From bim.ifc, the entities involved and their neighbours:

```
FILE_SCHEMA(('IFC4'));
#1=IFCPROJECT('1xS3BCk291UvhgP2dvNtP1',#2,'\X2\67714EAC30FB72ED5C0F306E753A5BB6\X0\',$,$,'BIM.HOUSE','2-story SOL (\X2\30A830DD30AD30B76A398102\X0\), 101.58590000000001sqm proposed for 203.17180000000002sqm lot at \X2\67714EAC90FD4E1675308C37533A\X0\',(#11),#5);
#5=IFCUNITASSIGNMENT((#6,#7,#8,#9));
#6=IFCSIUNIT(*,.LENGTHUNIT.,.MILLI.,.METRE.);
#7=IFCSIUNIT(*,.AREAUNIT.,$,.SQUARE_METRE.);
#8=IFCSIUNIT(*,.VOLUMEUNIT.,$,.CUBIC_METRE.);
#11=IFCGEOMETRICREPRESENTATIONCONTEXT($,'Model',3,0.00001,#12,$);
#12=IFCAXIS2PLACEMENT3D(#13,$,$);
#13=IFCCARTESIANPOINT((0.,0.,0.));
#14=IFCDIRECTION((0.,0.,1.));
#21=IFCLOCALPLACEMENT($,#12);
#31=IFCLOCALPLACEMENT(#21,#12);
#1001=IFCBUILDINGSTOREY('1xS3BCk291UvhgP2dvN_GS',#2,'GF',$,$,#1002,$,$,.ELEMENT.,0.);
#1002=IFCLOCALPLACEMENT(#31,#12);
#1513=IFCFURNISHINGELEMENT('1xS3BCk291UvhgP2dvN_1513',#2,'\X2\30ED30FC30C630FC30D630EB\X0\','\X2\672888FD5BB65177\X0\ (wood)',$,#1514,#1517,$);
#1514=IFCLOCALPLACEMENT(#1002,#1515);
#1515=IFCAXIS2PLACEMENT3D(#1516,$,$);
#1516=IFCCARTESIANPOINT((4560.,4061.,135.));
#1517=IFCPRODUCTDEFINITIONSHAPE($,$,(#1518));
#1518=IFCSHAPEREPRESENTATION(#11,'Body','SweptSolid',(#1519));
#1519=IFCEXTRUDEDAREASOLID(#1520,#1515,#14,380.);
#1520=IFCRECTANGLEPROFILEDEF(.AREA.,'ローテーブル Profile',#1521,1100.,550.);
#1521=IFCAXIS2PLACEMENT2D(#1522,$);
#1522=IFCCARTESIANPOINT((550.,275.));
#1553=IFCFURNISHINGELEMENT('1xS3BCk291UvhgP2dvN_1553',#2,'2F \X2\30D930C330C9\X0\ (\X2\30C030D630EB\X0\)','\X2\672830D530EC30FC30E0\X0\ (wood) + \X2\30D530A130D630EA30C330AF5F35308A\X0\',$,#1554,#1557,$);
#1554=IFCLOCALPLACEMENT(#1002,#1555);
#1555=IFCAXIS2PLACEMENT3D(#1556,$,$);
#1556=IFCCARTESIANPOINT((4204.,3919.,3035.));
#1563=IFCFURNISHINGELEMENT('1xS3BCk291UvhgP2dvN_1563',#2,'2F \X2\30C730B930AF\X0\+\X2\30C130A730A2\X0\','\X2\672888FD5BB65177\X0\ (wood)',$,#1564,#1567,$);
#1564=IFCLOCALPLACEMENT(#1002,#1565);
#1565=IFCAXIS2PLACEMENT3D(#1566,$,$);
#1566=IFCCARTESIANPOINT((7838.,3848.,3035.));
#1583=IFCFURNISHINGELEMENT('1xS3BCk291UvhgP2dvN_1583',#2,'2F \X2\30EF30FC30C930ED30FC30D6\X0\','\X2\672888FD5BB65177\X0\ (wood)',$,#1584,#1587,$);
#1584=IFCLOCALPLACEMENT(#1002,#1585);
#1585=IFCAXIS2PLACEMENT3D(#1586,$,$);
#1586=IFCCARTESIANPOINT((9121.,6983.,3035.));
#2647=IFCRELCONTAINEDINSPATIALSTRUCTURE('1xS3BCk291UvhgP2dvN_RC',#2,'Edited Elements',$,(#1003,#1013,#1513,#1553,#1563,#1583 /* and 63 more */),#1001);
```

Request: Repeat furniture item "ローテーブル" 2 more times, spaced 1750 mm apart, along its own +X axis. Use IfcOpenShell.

```python
import ifcopenshell
import ifcopenshell.api.geometry
import ifcopenshell.api.root
import ifcopenshell.util.element
import ifcopenshell.util.placement
import ifcopenshell.util.unit

model = ifcopenshell.open("bim.ifc")
unit_scale = ifcopenshell.util.unit.calculate_unit_scale(model)


def reuse_history(source, copy):
    """copy_class also copies each property set's owner history, people and application; keep the originals."""
    for rel in copy.IsDefinedBy:
        if rel.is_a("IfcRelDefinesByProperties") and (history := rel.RelatingPropertyDefinition.OwnerHistory):
            rel.RelatingPropertyDefinition.OwnerHistory = source.OwnerHistory
            ifcopenshell.util.element.remove_deep2(model, history)


source = model.by_guid("1xS3BCk291UvhgP2dvN_1513")
base = ifcopenshell.util.placement.get_local_placement(source.ObjectPlacement)
step = base[:3, 0] * 1.75 / unit_scale

for i in range(1, 3):
    copy = ifcopenshell.api.root.copy_class(model, product=source)
    copy.Representation = ifcopenshell.util.element.copy_deep(
        model, source.Representation, exclude=["IfcGeometricRepresentationContext", "IfcRepresentationMap"]
    )
    reuse_history(source, copy)
    matrix = base.copy()
    matrix[:3, 3] += i * step
    print("added at", matrix[:3, 3].round(3) + 0.0)
    ifcopenshell.api.geometry.edit_object_placement(model, product=copy, matrix=matrix, is_si=False)

model.write("bim_edited.ifc")
```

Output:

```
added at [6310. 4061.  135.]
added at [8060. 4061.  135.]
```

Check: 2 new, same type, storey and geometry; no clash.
